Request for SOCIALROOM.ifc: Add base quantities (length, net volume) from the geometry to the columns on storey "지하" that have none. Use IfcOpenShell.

First a look at what the model holds.

```python
import ifcopenshell
import ifcopenshell.util.element
import ifcopenshell.util.unit

model = ifcopenshell.open("SOCIALROOM.ifc")
print(model.schema)
for unit_type in ("LENGTHUNIT", "AREAUNIT", "VOLUMEUNIT"):
    print(unit_type, ifcopenshell.util.unit.calculate_unit_scale(model, unit_type))
storey = next(s for s in model.by_type("IfcBuildingStorey") if s.Name == "지하")
columns = [e for e in ifcopenshell.util.element.get_decomposition(storey) if e.is_a("IfcColumn")]
for e in sorted(columns, key=lambda e: e.id()):
    print(e.id(), e.is_a(), e.Name, list(ifcopenshell.util.element.get_psets(e, qtos_only=True)), sep=" | ")
```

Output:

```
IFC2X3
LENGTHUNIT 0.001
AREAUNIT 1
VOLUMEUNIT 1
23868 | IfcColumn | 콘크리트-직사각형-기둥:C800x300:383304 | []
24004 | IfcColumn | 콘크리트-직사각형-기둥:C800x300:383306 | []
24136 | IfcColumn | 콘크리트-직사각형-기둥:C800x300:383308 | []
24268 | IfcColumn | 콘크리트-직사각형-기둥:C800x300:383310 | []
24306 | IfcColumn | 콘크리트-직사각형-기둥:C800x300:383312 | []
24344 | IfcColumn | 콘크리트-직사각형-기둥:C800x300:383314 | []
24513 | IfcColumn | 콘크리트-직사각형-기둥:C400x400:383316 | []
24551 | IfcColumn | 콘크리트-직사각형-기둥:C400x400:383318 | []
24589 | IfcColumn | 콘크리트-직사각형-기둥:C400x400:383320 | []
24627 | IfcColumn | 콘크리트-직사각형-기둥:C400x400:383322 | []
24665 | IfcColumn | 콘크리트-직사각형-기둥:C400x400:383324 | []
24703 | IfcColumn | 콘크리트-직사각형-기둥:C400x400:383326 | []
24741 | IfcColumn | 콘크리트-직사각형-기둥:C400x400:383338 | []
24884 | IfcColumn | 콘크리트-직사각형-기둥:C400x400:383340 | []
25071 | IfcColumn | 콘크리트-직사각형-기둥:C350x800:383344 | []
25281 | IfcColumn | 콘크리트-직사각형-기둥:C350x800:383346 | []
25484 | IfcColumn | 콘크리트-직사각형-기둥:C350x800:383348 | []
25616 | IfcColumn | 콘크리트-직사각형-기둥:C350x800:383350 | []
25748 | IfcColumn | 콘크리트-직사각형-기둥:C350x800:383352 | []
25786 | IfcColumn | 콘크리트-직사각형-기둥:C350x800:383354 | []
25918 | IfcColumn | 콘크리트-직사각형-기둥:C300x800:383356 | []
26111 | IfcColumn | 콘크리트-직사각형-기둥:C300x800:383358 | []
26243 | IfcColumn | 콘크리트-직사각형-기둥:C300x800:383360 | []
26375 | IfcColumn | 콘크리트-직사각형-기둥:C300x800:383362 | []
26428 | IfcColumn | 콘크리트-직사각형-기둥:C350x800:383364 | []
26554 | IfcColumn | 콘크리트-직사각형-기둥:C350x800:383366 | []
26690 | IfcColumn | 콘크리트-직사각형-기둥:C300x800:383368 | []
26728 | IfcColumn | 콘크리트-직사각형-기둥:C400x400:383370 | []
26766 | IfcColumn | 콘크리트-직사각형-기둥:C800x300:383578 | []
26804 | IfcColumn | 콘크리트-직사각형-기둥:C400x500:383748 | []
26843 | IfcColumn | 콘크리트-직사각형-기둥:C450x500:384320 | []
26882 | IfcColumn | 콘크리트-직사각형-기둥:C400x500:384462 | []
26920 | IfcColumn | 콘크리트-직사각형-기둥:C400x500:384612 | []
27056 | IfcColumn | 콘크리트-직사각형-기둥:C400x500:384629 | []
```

```python
import ifcopenshell
import ifcopenshell.api.pset
import ifcopenshell.geom
import ifcopenshell.util.element
import ifcopenshell.util.shape
import ifcopenshell.util.unit

model = ifcopenshell.open("SOCIALROOM.ifc")
unit_scale = ifcopenshell.util.unit.calculate_unit_scale(model)
volume_scale = ifcopenshell.util.unit.calculate_unit_scale(model, "VOLUMEUNIT")
settings = ifcopenshell.geom.settings()

storey = next(s for s in model.by_type("IfcBuildingStorey") if s.Name == "지하")
columns = [e for e in ifcopenshell.util.element.get_decomposition(storey) if e.is_a("IfcColumn")]

for e in sorted(columns, key=lambda e: e.id()):
    if ifcopenshell.util.element.get_psets(e, qtos_only=True, should_inherit=False):
        continue
    # Geometry comes back in metres, in the element's own axes.
    shape = ifcopenshell.geom.create_shape(settings, e)
    values = {
        "Length": ifcopenshell.util.shape.get_z(shape.geometry) / unit_scale,
        "NetVolume": ifcopenshell.util.shape.get_volume(shape.geometry) / volume_scale,
    }
    qto = ifcopenshell.api.pset.add_qto(model, product=e, name="BaseQuantities")
    ifcopenshell.api.pset.edit_qto(model, qto=qto, properties=values)
    print(e.id(), {k: round(v, 3) for k, v in values.items()})

model.write("SOCIALROOM_edited.ifc")
```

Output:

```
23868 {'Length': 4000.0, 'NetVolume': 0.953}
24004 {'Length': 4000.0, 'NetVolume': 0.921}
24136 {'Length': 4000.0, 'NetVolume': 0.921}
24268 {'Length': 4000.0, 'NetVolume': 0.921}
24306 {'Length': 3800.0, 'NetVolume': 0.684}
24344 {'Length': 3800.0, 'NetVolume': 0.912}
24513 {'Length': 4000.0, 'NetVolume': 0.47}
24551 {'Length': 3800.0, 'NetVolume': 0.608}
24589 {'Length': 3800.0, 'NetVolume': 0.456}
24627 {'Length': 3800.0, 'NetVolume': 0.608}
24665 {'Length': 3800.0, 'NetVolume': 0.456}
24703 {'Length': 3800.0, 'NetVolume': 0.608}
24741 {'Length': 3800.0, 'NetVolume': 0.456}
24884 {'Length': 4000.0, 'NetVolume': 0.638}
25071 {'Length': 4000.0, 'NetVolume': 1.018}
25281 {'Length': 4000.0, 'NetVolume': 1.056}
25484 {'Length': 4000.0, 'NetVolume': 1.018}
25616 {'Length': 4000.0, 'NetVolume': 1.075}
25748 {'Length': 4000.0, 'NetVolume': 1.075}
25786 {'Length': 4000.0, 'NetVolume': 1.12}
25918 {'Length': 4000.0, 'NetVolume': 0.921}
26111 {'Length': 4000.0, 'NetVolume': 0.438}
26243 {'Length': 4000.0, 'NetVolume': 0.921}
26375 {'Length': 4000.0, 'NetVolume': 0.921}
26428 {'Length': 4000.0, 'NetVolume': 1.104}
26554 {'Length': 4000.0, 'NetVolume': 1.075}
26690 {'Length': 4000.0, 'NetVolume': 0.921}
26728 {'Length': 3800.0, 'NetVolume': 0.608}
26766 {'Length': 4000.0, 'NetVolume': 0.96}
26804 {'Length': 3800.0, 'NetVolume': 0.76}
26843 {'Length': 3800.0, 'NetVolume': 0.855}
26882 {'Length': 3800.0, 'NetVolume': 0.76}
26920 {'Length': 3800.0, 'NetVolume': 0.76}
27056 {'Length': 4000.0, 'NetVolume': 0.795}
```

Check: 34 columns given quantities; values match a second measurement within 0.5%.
